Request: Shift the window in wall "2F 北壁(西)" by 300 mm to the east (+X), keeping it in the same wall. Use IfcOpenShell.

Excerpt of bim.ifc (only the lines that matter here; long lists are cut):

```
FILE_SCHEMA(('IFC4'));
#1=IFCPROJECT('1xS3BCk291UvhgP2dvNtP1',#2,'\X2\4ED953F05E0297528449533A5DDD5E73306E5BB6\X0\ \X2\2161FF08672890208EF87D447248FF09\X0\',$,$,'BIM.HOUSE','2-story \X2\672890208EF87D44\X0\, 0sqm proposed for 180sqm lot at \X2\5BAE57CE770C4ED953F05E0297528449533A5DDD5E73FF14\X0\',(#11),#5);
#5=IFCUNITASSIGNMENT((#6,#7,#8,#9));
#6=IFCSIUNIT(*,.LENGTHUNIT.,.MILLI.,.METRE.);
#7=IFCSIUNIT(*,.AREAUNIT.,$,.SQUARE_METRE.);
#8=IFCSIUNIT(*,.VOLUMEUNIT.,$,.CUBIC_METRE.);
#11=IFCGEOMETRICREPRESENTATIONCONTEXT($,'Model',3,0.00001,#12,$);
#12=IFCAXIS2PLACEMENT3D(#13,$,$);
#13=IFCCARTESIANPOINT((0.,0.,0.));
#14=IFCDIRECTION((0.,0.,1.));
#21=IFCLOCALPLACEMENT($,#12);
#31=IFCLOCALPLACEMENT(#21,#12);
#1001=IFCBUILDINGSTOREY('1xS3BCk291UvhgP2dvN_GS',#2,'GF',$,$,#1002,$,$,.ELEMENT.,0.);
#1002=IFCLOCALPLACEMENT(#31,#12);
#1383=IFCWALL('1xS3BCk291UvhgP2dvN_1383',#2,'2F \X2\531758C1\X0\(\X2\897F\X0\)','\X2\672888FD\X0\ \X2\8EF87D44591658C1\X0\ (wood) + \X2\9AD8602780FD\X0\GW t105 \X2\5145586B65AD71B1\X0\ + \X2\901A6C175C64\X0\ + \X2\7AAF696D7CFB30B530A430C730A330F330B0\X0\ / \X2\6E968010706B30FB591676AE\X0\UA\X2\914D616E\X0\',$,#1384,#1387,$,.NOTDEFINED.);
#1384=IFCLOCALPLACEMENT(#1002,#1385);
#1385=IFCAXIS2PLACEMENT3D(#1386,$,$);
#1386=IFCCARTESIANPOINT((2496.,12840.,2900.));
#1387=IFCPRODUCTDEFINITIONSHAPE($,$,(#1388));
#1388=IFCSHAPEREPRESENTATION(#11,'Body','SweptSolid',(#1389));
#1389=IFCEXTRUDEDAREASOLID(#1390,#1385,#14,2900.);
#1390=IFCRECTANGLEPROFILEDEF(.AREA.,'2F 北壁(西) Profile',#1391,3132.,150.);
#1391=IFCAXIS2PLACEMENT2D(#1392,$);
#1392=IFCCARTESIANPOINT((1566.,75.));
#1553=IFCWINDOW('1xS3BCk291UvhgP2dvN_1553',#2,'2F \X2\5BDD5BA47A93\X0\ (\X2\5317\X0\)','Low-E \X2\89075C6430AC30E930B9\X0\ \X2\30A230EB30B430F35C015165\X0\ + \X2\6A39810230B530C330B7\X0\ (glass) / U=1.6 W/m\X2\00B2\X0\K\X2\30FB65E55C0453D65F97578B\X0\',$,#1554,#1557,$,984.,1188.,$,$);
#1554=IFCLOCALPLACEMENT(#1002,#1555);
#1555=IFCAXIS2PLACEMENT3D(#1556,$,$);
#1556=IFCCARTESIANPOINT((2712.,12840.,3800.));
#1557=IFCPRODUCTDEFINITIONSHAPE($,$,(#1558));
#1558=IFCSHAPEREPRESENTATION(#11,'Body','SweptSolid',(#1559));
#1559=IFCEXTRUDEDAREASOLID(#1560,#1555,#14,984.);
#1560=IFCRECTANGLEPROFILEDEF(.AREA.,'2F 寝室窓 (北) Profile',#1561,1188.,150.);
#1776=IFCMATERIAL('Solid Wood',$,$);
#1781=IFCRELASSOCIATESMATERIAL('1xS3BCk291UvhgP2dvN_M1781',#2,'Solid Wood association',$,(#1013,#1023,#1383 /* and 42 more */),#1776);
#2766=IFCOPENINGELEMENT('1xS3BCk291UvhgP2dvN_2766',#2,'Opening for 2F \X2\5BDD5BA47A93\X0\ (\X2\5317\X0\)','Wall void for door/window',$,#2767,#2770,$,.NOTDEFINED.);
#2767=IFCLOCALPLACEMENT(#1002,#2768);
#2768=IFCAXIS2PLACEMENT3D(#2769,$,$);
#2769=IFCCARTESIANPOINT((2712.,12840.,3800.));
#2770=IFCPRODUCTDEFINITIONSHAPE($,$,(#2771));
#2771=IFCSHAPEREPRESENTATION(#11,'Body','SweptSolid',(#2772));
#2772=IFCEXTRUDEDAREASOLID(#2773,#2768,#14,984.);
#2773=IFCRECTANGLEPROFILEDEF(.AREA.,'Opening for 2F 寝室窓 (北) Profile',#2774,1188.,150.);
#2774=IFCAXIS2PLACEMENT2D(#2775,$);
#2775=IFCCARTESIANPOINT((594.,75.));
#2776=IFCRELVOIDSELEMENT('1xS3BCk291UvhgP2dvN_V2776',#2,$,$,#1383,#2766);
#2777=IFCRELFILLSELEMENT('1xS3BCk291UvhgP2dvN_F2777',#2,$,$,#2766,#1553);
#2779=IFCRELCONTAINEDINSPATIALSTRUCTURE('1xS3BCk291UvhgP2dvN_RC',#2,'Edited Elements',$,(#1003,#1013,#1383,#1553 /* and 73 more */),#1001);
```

```python
import ifcopenshell
import ifcopenshell.api.geometry
import ifcopenshell.util.placement

model = ifcopenshell.open("bim.ifc")

window = model.by_id(1553)
opening = window.FillsVoids[0].RelatingOpeningElement
wall = opening.VoidsElements[0].RelatingBuildingElement

wall_matrix = ifcopenshell.util.placement.get_local_placement(wall.ObjectPlacement)
shift = wall_matrix[:3, 0] * 300.0
before = ifcopenshell.util.placement.get_local_placement(window.ObjectPlacement)[:3, 3].copy()

# The window is not placed relative to its opening, so move both.
for product in (opening, window):
    matrix = ifcopenshell.util.placement.get_local_placement(product.ObjectPlacement)
    matrix[:3, 3] += shift
    ifcopenshell.api.geometry.edit_object_placement(model, product=product, matrix=matrix, is_si=False)

after = ifcopenshell.util.placement.get_local_placement(window.ObjectPlacement)[:3, 3]
print("window moved by", (after - before).round(3) + 0.0)

model.write("bim_updated.ifc")
```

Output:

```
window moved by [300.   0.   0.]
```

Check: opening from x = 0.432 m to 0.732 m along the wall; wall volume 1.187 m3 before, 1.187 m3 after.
